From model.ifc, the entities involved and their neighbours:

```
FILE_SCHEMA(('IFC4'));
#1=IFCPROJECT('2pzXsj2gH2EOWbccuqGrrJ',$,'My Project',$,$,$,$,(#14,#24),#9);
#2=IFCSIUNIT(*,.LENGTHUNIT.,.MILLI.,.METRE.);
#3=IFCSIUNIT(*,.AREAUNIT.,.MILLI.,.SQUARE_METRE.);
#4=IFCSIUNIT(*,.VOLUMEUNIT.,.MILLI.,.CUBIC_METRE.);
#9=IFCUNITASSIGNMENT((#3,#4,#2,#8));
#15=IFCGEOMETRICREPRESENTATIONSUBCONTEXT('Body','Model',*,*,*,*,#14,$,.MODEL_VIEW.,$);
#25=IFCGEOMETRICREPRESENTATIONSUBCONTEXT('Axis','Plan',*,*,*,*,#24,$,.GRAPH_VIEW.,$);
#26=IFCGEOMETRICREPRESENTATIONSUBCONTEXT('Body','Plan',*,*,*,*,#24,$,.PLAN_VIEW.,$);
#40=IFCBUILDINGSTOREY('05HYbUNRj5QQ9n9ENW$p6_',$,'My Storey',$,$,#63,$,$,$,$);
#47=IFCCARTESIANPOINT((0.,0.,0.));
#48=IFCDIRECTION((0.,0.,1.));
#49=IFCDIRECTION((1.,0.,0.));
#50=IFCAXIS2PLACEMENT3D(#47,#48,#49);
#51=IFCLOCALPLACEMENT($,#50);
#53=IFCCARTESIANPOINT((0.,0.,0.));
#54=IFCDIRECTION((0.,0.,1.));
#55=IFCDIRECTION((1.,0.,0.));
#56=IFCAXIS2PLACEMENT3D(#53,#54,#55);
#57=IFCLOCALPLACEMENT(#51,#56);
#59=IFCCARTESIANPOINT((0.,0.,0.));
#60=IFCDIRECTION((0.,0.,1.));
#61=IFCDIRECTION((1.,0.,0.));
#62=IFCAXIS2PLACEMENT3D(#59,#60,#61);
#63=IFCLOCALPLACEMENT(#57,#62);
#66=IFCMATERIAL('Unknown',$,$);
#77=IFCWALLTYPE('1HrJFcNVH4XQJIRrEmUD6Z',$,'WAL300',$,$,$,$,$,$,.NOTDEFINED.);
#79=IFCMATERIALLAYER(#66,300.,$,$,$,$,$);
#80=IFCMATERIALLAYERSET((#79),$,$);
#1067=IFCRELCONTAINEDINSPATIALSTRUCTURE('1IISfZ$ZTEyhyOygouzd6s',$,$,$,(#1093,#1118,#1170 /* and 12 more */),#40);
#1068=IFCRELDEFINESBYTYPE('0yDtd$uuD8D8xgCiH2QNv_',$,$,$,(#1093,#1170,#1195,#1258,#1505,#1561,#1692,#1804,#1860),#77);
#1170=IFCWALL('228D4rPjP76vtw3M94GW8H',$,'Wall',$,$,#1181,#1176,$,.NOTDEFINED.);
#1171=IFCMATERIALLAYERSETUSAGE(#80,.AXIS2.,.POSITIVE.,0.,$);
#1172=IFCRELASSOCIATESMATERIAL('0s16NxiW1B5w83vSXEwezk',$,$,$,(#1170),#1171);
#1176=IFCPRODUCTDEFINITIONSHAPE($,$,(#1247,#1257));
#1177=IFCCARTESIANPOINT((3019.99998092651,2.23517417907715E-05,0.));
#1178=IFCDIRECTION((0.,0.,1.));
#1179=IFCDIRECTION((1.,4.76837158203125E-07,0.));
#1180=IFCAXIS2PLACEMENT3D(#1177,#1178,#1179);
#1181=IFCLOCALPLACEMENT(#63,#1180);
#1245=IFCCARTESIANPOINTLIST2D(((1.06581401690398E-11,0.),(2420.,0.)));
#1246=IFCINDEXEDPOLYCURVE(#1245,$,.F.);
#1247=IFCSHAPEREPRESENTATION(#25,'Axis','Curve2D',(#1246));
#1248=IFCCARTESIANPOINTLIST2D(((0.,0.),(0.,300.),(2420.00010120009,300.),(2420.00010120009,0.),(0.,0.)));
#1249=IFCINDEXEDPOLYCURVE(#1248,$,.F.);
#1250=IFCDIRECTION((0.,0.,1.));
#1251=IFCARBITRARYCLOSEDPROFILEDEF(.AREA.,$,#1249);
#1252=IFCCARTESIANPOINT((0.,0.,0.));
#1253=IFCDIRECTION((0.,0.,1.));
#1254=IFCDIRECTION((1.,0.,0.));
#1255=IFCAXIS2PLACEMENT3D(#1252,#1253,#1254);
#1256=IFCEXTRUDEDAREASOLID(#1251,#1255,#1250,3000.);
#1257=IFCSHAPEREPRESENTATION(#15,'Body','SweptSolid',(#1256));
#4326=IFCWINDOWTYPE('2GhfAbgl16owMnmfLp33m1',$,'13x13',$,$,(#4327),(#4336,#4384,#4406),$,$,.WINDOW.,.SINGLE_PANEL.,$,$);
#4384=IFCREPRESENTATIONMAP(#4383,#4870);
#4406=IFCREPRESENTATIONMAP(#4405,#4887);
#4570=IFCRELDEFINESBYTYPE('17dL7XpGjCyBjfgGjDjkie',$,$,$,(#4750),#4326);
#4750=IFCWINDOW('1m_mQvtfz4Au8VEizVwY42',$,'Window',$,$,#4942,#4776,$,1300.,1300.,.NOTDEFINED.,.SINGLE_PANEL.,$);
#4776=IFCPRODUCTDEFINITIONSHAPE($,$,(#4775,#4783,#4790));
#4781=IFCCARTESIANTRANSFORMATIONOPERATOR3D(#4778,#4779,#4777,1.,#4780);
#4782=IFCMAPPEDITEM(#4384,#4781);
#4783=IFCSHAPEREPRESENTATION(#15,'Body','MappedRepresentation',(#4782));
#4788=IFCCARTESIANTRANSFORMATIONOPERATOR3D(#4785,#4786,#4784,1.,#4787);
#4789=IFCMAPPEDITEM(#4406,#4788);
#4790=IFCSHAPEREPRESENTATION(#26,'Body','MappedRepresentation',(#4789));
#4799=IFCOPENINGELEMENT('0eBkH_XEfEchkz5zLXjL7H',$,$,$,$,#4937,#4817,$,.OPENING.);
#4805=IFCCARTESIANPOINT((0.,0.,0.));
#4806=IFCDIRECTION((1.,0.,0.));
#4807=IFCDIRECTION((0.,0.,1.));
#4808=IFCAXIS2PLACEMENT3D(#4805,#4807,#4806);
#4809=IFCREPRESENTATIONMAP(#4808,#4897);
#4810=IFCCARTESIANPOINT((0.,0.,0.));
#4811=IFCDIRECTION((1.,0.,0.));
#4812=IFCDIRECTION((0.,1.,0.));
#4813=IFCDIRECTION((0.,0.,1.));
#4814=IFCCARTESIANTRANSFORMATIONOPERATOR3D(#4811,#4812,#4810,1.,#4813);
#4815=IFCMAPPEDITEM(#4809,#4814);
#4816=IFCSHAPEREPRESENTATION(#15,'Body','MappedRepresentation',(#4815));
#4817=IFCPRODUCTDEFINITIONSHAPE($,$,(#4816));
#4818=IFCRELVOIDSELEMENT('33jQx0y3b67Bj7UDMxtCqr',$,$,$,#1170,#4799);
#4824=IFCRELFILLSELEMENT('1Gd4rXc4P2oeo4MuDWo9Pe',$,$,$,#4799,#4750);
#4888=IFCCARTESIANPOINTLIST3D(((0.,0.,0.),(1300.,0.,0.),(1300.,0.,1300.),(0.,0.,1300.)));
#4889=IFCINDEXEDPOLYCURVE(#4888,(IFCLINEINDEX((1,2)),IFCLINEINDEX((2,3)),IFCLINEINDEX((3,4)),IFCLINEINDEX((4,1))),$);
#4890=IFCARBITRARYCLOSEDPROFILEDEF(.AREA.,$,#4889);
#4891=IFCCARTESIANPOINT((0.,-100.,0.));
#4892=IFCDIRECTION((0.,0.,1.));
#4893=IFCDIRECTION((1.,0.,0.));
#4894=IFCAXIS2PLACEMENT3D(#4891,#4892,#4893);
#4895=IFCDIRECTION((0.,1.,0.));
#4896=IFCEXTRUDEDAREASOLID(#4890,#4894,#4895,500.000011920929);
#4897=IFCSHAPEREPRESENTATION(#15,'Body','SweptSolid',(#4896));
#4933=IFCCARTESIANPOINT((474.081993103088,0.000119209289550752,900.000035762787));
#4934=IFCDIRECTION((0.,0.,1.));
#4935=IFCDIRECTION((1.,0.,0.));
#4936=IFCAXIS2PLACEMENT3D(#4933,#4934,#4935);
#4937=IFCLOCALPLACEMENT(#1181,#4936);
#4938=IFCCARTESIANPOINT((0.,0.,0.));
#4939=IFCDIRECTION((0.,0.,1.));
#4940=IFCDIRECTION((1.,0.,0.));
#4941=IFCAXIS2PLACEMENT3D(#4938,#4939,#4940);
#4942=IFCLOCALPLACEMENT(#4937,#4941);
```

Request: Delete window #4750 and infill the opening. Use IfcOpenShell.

```python
import ifcopenshell
import ifcopenshell.api.feature
import ifcopenshell.api.root
import ifcopenshell.geom
import ifcopenshell.util.shape

model = ifcopenshell.open("model.ifc")
settings = ifcopenshell.geom.settings()


def volume(element):
    """Net volume in cubic metres, openings subtracted."""
    shape = ifcopenshell.geom.create_shape(settings, element)
    return ifcopenshell.util.shape.get_volume(shape.geometry)


window = model.by_guid("1m_mQvtfz4Au8VEizVwY42")
opening = window.FillsVoids[0].RelatingOpeningElement
wall = opening.VoidsElements[0].RelatingBuildingElement
before = volume(wall)

ifcopenshell.api.root.remove_product(model, product=window)
ifcopenshell.api.feature.remove_feature(model, feature=opening)

after = volume(wall)

print(f"wall volume {before:.3f} -> {after:.3f} m3")

model.write("model_edited.ifc")
```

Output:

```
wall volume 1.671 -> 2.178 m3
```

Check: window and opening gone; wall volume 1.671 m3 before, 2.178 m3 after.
